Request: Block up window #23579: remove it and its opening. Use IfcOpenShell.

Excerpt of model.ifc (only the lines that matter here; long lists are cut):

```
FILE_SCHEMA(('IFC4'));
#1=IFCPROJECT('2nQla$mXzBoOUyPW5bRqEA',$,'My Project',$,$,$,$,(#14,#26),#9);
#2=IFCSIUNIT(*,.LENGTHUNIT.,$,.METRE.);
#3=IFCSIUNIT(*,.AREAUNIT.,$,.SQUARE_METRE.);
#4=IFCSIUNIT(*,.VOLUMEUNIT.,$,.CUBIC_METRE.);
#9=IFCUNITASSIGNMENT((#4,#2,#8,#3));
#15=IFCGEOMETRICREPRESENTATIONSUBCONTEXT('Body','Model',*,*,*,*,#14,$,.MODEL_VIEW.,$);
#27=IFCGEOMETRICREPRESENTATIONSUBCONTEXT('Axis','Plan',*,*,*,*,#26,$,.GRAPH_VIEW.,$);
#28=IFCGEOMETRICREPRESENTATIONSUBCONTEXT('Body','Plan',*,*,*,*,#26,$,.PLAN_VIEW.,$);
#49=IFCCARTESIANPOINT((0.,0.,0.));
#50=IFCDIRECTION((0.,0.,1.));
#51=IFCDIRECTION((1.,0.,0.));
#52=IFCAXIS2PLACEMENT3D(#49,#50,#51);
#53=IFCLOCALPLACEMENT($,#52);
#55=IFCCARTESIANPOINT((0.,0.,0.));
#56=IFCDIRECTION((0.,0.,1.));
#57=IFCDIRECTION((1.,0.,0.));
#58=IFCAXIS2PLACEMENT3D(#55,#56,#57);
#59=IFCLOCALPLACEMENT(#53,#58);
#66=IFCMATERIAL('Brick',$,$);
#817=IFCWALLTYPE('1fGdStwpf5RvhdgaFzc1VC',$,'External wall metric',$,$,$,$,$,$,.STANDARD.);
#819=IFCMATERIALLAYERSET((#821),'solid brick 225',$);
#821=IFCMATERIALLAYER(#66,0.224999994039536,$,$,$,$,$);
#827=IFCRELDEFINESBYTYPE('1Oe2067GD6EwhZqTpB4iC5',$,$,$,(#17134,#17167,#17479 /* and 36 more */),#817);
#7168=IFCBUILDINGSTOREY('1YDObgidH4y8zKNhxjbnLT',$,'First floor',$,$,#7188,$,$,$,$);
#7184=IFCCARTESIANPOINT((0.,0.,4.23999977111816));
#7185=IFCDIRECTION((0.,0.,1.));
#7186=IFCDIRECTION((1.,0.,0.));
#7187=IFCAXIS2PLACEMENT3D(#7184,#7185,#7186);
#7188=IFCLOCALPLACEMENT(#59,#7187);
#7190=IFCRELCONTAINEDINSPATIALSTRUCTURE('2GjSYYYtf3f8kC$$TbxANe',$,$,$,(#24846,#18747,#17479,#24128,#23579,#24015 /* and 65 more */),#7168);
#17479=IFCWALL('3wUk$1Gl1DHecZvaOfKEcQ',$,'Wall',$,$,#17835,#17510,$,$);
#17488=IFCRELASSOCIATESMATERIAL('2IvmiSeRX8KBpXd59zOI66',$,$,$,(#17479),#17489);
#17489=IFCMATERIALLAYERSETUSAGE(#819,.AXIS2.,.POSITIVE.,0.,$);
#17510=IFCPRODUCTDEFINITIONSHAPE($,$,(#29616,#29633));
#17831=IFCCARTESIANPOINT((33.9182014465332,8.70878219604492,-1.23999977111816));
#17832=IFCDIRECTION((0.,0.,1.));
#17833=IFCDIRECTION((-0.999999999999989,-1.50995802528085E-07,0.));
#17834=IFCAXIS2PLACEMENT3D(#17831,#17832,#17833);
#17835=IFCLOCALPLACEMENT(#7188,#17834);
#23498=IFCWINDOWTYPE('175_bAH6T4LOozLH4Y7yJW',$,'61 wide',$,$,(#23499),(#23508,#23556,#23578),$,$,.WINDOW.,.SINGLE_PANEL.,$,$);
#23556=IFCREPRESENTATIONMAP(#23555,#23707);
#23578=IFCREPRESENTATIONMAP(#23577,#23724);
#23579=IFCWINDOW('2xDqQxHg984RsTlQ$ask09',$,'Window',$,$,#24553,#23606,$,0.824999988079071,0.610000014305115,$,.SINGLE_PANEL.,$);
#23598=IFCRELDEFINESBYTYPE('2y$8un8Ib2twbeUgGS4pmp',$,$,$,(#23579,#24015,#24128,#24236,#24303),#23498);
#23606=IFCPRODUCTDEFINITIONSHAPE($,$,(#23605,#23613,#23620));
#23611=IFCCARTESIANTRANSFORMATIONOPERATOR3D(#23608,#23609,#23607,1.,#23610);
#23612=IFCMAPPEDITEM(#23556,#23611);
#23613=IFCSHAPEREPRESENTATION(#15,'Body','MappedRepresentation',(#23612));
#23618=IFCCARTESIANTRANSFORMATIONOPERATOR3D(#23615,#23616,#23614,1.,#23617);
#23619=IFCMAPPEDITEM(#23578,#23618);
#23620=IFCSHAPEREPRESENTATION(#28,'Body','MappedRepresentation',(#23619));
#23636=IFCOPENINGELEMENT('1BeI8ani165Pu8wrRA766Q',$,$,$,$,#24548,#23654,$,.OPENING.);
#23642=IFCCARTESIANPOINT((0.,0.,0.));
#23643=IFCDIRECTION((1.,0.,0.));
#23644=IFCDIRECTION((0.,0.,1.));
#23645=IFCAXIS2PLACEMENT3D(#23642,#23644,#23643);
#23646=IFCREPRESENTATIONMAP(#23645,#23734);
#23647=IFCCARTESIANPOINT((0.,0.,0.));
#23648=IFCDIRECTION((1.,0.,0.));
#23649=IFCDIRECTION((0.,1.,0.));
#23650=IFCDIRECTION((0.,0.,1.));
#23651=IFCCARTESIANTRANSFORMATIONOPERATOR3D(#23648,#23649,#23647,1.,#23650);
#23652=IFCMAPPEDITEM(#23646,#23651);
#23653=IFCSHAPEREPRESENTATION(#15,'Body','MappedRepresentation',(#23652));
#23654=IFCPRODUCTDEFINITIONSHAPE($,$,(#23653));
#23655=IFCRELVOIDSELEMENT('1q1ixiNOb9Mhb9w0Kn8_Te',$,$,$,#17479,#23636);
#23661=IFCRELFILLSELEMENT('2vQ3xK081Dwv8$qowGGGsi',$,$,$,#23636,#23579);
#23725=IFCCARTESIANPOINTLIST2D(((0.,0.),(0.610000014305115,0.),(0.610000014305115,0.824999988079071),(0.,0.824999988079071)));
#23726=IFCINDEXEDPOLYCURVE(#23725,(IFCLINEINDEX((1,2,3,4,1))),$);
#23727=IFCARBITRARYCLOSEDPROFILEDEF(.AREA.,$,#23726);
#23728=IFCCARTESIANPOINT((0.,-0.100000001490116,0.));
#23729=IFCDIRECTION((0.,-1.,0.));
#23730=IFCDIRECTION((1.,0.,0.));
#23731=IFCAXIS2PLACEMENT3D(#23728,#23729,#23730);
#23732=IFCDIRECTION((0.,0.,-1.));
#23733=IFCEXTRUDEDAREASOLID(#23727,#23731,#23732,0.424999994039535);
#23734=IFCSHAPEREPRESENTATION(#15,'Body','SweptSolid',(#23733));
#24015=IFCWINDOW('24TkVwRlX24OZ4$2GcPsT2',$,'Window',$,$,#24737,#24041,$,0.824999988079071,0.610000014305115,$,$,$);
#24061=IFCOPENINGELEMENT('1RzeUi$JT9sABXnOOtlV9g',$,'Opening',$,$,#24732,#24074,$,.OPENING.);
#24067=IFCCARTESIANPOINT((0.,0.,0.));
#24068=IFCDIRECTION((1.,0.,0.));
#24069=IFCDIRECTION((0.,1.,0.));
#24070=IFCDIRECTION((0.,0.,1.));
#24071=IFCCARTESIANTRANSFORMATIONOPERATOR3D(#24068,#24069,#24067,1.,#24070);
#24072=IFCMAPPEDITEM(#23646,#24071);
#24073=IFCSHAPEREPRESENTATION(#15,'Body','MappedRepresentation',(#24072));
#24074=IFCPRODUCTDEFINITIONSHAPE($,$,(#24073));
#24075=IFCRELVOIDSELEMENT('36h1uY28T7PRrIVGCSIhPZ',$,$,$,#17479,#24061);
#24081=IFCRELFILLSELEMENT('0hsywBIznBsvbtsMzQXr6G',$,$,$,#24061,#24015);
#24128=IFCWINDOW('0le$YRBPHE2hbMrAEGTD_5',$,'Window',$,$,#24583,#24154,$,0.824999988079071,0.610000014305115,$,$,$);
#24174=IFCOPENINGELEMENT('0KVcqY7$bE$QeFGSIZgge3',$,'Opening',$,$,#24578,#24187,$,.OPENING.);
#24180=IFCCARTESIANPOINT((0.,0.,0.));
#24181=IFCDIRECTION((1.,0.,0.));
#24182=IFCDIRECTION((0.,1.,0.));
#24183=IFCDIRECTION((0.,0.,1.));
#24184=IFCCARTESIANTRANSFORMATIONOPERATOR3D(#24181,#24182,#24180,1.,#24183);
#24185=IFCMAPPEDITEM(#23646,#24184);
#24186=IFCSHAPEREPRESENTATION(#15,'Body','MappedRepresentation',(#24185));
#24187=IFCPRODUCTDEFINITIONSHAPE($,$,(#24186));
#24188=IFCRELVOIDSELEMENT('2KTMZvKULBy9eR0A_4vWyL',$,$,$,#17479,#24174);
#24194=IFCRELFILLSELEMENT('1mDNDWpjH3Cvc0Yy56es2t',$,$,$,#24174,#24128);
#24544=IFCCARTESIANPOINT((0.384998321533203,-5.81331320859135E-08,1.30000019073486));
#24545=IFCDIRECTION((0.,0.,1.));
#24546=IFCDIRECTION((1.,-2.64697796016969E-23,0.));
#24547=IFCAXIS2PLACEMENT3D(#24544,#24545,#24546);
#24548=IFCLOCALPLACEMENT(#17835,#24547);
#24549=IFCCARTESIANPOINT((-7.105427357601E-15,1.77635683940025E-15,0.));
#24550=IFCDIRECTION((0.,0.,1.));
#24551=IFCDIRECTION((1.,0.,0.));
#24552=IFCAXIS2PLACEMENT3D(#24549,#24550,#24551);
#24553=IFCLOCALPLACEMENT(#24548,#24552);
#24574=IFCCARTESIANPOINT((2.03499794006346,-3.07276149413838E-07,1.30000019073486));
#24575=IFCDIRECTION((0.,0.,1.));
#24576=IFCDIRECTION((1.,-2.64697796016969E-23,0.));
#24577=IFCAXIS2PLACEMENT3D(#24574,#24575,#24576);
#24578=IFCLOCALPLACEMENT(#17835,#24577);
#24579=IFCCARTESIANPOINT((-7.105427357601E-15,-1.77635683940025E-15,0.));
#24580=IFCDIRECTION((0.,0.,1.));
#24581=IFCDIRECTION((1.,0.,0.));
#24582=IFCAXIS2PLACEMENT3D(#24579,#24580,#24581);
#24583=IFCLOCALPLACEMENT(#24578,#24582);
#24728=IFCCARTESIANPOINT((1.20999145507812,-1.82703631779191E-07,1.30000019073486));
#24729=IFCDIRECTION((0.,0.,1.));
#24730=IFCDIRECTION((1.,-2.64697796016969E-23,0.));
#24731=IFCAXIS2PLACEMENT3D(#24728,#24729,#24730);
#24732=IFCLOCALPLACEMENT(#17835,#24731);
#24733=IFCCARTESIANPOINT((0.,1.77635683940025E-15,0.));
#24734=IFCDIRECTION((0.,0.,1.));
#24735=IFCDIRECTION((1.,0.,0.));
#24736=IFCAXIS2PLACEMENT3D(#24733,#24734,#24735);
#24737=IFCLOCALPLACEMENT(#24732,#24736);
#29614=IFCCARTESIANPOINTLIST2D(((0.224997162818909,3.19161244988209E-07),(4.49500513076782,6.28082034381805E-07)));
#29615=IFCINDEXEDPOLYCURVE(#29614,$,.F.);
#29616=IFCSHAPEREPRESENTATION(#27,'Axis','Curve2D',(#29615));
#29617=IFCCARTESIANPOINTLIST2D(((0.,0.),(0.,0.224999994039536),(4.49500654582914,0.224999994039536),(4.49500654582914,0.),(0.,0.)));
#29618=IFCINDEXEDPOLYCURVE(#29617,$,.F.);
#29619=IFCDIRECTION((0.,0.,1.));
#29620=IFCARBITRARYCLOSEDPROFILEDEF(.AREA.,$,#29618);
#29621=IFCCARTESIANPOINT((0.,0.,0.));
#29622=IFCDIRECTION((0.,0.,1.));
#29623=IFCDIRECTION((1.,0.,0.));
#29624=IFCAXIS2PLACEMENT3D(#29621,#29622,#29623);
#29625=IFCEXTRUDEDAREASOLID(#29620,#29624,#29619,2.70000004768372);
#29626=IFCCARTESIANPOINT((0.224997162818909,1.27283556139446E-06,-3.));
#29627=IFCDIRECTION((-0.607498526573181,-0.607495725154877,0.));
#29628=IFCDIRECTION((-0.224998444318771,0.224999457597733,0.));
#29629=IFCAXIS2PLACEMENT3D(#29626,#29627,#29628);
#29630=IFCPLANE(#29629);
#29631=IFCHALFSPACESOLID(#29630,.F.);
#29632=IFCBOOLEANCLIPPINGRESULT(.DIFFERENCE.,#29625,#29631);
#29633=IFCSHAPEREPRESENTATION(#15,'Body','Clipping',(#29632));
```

```python
import ifcopenshell
import ifcopenshell.api.feature
import ifcopenshell.api.root
import ifcopenshell.geom
import ifcopenshell.util.shape

model = ifcopenshell.open("model.ifc")
settings = ifcopenshell.geom.settings()


def volume(element):
    """Net volume in cubic metres, openings subtracted."""
    shape = ifcopenshell.geom.create_shape(settings, element)
    return ifcopenshell.util.shape.get_volume(shape.geometry)


window = model.by_id(23579)
opening = window.FillsVoids[0].RelatingOpeningElement
wall = opening.VoidsElements[0].RelatingBuildingElement
before = volume(wall)

ifcopenshell.api.root.remove_product(model, product=window)
ifcopenshell.api.feature.remove_feature(model, feature=opening)

after = volume(wall)

print(f"wall volume {before:.3f} -> {after:.3f} m3")

model.write("model_rev.ifc")
```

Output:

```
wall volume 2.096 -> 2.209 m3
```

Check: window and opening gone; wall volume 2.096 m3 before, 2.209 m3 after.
